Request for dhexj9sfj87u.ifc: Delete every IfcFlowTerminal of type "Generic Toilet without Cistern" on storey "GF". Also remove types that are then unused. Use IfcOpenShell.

First a look at what the model holds.

```python
import ifcopenshell
import ifcopenshell.util.element

model = ifcopenshell.open("dhexj9sfj87u.ifc")
print(model.schema)
storey = next(s for s in model.by_type("IfcBuildingStorey") if s.Name == "GF")
terminals = [e for e in ifcopenshell.util.element.get_decomposition(storey) if e.is_a("IfcFlowTerminal")]
seen = {}
for e in terminals:
    element_type = ifcopenshell.util.element.get_type(e)
    name = element_type.Name if element_type not in (None, e) else None
    seen[name] = seen.get(name, 0) + 1
for name, count in sorted(seen.items(), key=str):
    print(count, "x", name)
```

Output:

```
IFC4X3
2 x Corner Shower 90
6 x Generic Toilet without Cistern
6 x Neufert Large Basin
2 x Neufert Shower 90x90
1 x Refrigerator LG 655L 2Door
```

```python
import ifcopenshell
import ifcopenshell.api.root
import ifcopenshell.util.element

model = ifcopenshell.open("dhexj9sfj87u.ifc")

storey = next(s for s in model.by_type("IfcBuildingStorey") if s.Name == "GF")
terminals = [e for e in ifcopenshell.util.element.get_decomposition(storey) if e.is_a("IfcFlowTerminal")]
targets = [e for e in terminals if (t := ifcopenshell.util.element.get_type(e)) not in (None, e) and t.Name == "Generic Toilet without Cistern"]
types = {ifcopenshell.util.element.get_type(e) for e in targets} - {None, *targets}

for e in targets:
    ifcopenshell.api.root.remove_product(model, product=e)
print(len(targets), "removed")

unused = [t for t in types if not ifcopenshell.util.element.get_types(t)]
for t in unused:
    ifcopenshell.api.root.remove_product(model, product=t)
print(len(unused), "unused types removed")

model.write("dhexj9sfj87u-out.ifc")
```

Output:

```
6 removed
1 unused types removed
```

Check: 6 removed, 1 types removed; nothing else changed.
